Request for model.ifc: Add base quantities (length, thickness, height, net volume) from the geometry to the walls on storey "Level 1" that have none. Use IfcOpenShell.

First a look at what the model holds.

```python
import ifcopenshell
import ifcopenshell.util.element
import ifcopenshell.util.unit

model = ifcopenshell.open("model.ifc")
print(model.schema)
for unit_type in ("LENGTHUNIT", "AREAUNIT", "VOLUMEUNIT"):
    print(unit_type, ifcopenshell.util.unit.calculate_unit_scale(model, unit_type))
storey = next(s for s in model.by_type("IfcBuildingStorey") if s.Name == "Level 1")
walls = [e for e in ifcopenshell.util.element.get_decomposition(storey) if e.is_a("IfcWall")]
for e in sorted(walls, key=lambda e: e.id()):
    print(e.id(), e.is_a(), e.Name, list(ifcopenshell.util.element.get_psets(e, qtos_only=True)), sep=" | ")
```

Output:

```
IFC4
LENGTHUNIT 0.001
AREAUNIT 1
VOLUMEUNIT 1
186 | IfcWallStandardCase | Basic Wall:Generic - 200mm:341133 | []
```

```python
import ifcopenshell
import ifcopenshell.api.pset
import ifcopenshell.geom
import ifcopenshell.util.element
import ifcopenshell.util.shape
import ifcopenshell.util.unit

model = ifcopenshell.open("model.ifc")
unit_scale = ifcopenshell.util.unit.calculate_unit_scale(model)
volume_scale = ifcopenshell.util.unit.calculate_unit_scale(model, "VOLUMEUNIT")
settings = ifcopenshell.geom.settings()

storey = next(s for s in model.by_type("IfcBuildingStorey") if s.Name == "Level 1")
walls = [e for e in ifcopenshell.util.element.get_decomposition(storey) if e.is_a("IfcWall")]

for e in sorted(walls, key=lambda e: e.id()):
    if ifcopenshell.util.element.get_psets(e, qtos_only=True, should_inherit=False):
        continue
    # Geometry comes back in metres, in the element's own axes.
    shape = ifcopenshell.geom.create_shape(settings, e)
    values = {
        "Length": ifcopenshell.util.shape.get_x(shape.geometry) / unit_scale,
        "Width": ifcopenshell.util.shape.get_y(shape.geometry) / unit_scale,
        "Height": ifcopenshell.util.shape.get_z(shape.geometry) / unit_scale,
        "NetVolume": ifcopenshell.util.shape.get_volume(shape.geometry) / volume_scale,
    }
    qto = ifcopenshell.api.pset.add_qto(model, product=e, name="Qto_WallBaseQuantities")
    ifcopenshell.api.pset.edit_qto(model, qto=qto, properties=values)
    print(e.id(), {k: round(v, 3) for k, v in values.items()})

model.write("model_rev.ifc")
```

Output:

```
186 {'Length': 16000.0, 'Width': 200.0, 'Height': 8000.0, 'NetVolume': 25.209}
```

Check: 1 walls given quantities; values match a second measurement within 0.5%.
